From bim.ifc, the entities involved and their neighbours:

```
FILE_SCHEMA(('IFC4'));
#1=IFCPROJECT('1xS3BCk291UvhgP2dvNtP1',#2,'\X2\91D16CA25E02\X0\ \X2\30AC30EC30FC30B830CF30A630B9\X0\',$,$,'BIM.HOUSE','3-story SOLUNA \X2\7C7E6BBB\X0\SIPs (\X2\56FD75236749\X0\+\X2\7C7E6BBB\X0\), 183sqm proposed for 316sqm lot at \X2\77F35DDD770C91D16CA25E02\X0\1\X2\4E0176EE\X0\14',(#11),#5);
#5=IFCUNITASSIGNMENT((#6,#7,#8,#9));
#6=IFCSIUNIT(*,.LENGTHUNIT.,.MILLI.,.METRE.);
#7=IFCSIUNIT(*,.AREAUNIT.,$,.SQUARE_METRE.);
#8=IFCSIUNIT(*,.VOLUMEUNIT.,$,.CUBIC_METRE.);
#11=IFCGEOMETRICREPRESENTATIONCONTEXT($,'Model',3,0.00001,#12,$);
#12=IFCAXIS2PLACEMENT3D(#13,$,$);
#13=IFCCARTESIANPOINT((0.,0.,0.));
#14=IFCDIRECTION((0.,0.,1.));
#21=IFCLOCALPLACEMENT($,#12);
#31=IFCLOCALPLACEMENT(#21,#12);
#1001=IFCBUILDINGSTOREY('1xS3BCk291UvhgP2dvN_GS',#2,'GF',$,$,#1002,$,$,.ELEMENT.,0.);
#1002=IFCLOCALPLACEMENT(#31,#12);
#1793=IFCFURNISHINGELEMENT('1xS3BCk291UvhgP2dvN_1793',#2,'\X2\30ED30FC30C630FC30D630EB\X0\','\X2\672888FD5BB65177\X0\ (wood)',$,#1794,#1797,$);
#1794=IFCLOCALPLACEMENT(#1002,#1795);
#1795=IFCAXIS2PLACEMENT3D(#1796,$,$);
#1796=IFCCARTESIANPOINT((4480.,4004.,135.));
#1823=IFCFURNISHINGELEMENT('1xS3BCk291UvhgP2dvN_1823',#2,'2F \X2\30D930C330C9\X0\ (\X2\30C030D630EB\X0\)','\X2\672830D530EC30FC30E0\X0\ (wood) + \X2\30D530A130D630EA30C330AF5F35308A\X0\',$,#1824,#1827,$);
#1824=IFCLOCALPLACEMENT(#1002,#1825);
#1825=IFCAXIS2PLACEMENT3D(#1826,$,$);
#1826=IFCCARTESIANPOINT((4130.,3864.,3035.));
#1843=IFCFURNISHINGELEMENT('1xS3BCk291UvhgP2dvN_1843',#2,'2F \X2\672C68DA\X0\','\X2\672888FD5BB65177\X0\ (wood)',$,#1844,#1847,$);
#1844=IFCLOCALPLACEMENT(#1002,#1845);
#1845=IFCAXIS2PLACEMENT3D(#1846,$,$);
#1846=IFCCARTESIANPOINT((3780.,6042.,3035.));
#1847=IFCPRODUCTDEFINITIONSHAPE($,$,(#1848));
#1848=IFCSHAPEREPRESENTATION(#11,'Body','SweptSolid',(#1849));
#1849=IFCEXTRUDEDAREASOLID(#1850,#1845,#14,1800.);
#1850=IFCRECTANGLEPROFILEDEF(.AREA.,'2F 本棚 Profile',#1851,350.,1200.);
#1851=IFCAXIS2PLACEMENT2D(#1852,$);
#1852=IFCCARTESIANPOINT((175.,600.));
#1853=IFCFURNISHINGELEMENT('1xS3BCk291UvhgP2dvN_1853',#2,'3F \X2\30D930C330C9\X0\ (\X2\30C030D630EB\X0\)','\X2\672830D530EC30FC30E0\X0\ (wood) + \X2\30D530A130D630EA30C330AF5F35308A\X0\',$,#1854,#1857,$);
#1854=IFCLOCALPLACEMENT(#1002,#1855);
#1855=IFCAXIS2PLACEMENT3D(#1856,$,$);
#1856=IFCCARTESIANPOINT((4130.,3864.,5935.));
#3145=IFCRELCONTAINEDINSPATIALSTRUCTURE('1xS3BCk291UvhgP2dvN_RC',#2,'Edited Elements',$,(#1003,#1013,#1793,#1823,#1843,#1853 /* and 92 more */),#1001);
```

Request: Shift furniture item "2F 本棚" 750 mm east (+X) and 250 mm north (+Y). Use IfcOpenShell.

```python
import ifcopenshell
import ifcopenshell.api.geometry
import ifcopenshell.util.placement

model = ifcopenshell.open("bim.ifc")

item = model.by_id(1843)
matrix = ifcopenshell.util.placement.get_local_placement(item.ObjectPlacement)
matrix[0, 3] += 750.0
matrix[1, 3] += 250.0
ifcopenshell.api.geometry.edit_object_placement(model, product=item, matrix=matrix, is_si=False)

print(ifcopenshell.util.placement.get_local_placement(item.ObjectPlacement).round(3) + 0.0)

model.write("bim_edited.ifc")
```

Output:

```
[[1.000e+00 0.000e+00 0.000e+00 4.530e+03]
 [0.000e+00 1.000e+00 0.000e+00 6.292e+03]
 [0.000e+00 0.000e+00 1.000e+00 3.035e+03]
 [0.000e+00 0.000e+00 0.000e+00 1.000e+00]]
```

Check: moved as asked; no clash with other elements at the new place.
